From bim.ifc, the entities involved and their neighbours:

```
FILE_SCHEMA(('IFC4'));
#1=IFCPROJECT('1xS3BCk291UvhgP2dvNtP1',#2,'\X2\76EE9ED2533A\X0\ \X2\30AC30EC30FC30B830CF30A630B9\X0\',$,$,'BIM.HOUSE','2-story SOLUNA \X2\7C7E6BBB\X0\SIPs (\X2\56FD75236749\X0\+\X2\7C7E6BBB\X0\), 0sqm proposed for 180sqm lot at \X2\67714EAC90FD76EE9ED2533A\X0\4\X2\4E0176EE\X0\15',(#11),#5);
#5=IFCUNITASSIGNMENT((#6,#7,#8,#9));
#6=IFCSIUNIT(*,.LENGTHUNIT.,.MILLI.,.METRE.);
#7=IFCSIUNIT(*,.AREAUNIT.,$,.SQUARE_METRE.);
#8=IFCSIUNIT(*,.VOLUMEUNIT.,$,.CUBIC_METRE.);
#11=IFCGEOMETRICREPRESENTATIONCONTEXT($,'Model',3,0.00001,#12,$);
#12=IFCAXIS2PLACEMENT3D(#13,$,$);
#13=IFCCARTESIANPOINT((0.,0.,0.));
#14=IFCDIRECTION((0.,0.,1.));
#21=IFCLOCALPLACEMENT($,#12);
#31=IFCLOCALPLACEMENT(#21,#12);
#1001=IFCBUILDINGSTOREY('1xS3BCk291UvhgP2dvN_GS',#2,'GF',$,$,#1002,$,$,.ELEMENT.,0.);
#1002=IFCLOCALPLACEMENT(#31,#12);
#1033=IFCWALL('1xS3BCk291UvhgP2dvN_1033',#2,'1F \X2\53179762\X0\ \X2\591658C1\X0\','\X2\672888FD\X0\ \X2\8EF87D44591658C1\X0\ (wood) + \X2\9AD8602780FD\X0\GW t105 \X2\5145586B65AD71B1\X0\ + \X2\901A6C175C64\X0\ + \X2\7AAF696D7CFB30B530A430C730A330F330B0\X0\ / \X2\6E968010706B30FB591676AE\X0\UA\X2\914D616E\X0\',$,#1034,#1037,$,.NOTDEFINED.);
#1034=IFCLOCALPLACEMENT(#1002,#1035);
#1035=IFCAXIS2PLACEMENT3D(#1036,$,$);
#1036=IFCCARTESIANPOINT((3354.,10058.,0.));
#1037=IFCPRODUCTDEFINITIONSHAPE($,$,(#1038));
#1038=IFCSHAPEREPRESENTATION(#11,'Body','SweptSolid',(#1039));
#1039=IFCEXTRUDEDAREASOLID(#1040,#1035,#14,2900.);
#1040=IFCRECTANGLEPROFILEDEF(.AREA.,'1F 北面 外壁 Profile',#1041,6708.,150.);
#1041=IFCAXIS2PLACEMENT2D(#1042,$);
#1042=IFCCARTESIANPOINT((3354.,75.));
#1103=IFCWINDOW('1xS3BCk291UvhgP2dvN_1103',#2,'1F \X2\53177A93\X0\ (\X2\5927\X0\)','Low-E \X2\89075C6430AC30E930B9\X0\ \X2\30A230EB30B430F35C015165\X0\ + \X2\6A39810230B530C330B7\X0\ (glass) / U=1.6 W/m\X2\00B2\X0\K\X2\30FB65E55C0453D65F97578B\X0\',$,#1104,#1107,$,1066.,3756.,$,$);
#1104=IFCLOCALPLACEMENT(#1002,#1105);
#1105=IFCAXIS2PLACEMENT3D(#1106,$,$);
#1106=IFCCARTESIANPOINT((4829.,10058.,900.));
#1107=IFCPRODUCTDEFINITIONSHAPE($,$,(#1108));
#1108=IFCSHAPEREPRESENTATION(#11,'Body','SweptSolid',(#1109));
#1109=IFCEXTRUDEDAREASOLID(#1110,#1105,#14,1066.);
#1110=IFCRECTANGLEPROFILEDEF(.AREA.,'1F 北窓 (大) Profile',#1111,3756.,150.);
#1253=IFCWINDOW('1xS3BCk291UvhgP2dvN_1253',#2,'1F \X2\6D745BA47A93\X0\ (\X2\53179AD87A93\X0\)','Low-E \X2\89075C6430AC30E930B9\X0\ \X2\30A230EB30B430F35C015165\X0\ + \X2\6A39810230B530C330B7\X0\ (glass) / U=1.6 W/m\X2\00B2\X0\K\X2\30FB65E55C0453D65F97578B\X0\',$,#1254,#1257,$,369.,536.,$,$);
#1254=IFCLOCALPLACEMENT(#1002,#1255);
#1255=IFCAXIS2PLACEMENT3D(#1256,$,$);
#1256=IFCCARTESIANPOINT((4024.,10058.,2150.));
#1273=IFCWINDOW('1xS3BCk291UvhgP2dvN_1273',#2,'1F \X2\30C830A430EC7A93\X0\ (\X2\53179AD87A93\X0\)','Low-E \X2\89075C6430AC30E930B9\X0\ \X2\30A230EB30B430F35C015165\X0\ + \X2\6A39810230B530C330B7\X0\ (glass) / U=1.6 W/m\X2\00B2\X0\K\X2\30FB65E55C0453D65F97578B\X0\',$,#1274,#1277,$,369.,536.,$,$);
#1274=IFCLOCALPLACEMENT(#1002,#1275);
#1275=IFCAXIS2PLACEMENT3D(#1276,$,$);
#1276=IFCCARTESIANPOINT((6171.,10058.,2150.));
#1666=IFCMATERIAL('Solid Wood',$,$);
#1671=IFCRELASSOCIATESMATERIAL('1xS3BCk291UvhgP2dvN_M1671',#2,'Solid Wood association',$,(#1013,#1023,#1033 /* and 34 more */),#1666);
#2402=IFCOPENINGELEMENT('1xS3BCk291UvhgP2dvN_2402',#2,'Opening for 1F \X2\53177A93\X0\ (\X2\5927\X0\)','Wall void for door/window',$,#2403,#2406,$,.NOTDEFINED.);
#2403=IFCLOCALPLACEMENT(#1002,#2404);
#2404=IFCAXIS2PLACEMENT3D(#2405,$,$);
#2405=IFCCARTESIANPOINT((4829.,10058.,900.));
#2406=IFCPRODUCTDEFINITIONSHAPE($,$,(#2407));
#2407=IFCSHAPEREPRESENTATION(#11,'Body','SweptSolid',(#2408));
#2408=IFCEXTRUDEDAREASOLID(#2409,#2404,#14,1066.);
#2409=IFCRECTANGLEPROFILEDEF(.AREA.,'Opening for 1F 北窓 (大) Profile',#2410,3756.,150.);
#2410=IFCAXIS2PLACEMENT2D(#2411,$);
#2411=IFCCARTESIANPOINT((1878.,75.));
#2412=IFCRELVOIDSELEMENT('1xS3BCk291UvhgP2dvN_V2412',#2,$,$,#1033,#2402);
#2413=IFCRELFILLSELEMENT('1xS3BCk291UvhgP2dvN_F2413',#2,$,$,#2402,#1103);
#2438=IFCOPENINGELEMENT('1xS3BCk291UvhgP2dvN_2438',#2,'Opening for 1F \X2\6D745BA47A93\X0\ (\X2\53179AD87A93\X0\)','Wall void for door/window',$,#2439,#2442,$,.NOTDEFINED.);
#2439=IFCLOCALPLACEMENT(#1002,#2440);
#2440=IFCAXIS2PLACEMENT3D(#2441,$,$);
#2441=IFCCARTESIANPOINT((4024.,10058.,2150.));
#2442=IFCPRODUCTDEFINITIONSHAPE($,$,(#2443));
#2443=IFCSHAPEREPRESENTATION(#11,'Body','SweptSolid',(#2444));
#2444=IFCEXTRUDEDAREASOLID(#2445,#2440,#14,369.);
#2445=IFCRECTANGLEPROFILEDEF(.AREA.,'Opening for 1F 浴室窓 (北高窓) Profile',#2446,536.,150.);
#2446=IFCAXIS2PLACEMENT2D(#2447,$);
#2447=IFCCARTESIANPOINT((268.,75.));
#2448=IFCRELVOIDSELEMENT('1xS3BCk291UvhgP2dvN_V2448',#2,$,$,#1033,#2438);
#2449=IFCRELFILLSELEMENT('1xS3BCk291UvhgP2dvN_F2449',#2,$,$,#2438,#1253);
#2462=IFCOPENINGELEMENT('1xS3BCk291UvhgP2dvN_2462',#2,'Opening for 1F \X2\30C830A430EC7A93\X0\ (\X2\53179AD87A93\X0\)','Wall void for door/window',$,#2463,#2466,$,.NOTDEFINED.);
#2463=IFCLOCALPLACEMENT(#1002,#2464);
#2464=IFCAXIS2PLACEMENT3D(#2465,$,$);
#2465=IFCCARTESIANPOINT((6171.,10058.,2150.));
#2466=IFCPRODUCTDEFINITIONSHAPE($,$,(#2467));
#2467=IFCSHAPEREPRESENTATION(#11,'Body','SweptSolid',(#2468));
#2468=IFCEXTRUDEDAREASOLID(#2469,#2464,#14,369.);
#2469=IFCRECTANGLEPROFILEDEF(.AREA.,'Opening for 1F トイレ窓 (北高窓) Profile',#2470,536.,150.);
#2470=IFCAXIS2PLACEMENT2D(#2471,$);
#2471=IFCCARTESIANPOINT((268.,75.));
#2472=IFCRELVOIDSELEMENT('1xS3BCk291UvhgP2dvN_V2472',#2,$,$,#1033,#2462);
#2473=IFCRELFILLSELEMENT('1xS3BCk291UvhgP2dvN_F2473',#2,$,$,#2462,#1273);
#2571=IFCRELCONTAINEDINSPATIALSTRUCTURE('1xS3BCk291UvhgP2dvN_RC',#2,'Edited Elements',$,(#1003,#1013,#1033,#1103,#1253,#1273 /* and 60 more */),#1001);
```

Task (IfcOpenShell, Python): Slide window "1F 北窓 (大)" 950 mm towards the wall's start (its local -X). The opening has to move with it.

```python
import ifcopenshell
import ifcopenshell.api.geometry
import ifcopenshell.util.placement
import ifcopenshell.util.unit

model = ifcopenshell.open("bim.ifc")
unit_scale = ifcopenshell.util.unit.calculate_unit_scale(model)

window = model.by_guid("1xS3BCk291UvhgP2dvN_1103")
opening = window.FillsVoids[0].RelatingOpeningElement
wall = opening.VoidsElements[0].RelatingBuildingElement

wall_matrix = ifcopenshell.util.placement.get_local_placement(wall.ObjectPlacement)
shift = wall_matrix[:3, 0] * -0.95 / unit_scale
before = ifcopenshell.util.placement.get_local_placement(window.ObjectPlacement)[:3, 3].copy()

# The window is not placed relative to its opening, so move both.
for product in (opening, window):
    matrix = ifcopenshell.util.placement.get_local_placement(product.ObjectPlacement)
    matrix[:3, 3] += shift
    ifcopenshell.api.geometry.edit_object_placement(model, product=product, matrix=matrix, is_si=False)

after = ifcopenshell.util.placement.get_local_placement(window.ObjectPlacement)[:3, 3]
print("window moved by", (after - before).round(3) + 0.0)

model.write("bim_v2.ifc")
```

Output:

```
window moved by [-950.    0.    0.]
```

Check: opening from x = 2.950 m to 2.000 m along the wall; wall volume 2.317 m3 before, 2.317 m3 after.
